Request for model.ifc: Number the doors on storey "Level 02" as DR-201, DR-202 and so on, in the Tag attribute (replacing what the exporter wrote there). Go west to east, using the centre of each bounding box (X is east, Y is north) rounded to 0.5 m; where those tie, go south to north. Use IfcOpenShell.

First a look at what the model holds.

```python
import ifcopenshell
import ifcopenshell.util.element
import ifcopenshell.util.placement

model = ifcopenshell.open("model.ifc")
print(model.schema)
storey = next(s for s in model.by_type("IfcBuildingStorey") if s.Name == "Level 02")
doors = [e for e in ifcopenshell.util.element.get_decomposition(storey) if e.is_a("IfcDoor")]
for e in sorted(doors, key=lambda e: e.id()):
    origin = ifcopenshell.util.placement.get_local_placement(e.ObjectPlacement)[:3, 3]
    print(e.id(), e.Tag, e.Name, origin.round(2) + 0.0, sep=" | ")
```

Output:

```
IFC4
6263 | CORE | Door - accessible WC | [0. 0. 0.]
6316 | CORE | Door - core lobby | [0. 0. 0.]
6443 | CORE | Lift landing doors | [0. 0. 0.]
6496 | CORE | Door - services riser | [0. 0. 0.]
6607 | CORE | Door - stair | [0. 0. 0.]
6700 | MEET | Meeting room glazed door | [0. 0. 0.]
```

```python
import ifcopenshell
import ifcopenshell.geom
import ifcopenshell.util.element
import ifcopenshell.util.shape

model = ifcopenshell.open("model.ifc")
settings = ifcopenshell.geom.settings()
settings.set("use-world-coords", True)


def centre(element):
    shape = ifcopenshell.geom.create_shape(settings, element)
    return ifcopenshell.util.shape.get_bbox_centroid(shape.geometry)


storey = next(s for s in model.by_type("IfcBuildingStorey") if s.Name == "Level 02")
doors = [e for e in ifcopenshell.util.element.get_decomposition(storey) if e.is_a("IfcDoor")]

# Insertion points can sit at a corner or the storey origin, so sort by the geometry (in metres).
centres = {e: centre(e) for e in doors}
doors.sort(key=lambda e: (round(centres[e][0] / 0.5), centres[e][1]))

for i, e in enumerate(doors, start=1):
    number = f"DR-2{i:02d}"
    e.Tag = number
    print(e.id(), number)

model.write("model_edited.ifc")
```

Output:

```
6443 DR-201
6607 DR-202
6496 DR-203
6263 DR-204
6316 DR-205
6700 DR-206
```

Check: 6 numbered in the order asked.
